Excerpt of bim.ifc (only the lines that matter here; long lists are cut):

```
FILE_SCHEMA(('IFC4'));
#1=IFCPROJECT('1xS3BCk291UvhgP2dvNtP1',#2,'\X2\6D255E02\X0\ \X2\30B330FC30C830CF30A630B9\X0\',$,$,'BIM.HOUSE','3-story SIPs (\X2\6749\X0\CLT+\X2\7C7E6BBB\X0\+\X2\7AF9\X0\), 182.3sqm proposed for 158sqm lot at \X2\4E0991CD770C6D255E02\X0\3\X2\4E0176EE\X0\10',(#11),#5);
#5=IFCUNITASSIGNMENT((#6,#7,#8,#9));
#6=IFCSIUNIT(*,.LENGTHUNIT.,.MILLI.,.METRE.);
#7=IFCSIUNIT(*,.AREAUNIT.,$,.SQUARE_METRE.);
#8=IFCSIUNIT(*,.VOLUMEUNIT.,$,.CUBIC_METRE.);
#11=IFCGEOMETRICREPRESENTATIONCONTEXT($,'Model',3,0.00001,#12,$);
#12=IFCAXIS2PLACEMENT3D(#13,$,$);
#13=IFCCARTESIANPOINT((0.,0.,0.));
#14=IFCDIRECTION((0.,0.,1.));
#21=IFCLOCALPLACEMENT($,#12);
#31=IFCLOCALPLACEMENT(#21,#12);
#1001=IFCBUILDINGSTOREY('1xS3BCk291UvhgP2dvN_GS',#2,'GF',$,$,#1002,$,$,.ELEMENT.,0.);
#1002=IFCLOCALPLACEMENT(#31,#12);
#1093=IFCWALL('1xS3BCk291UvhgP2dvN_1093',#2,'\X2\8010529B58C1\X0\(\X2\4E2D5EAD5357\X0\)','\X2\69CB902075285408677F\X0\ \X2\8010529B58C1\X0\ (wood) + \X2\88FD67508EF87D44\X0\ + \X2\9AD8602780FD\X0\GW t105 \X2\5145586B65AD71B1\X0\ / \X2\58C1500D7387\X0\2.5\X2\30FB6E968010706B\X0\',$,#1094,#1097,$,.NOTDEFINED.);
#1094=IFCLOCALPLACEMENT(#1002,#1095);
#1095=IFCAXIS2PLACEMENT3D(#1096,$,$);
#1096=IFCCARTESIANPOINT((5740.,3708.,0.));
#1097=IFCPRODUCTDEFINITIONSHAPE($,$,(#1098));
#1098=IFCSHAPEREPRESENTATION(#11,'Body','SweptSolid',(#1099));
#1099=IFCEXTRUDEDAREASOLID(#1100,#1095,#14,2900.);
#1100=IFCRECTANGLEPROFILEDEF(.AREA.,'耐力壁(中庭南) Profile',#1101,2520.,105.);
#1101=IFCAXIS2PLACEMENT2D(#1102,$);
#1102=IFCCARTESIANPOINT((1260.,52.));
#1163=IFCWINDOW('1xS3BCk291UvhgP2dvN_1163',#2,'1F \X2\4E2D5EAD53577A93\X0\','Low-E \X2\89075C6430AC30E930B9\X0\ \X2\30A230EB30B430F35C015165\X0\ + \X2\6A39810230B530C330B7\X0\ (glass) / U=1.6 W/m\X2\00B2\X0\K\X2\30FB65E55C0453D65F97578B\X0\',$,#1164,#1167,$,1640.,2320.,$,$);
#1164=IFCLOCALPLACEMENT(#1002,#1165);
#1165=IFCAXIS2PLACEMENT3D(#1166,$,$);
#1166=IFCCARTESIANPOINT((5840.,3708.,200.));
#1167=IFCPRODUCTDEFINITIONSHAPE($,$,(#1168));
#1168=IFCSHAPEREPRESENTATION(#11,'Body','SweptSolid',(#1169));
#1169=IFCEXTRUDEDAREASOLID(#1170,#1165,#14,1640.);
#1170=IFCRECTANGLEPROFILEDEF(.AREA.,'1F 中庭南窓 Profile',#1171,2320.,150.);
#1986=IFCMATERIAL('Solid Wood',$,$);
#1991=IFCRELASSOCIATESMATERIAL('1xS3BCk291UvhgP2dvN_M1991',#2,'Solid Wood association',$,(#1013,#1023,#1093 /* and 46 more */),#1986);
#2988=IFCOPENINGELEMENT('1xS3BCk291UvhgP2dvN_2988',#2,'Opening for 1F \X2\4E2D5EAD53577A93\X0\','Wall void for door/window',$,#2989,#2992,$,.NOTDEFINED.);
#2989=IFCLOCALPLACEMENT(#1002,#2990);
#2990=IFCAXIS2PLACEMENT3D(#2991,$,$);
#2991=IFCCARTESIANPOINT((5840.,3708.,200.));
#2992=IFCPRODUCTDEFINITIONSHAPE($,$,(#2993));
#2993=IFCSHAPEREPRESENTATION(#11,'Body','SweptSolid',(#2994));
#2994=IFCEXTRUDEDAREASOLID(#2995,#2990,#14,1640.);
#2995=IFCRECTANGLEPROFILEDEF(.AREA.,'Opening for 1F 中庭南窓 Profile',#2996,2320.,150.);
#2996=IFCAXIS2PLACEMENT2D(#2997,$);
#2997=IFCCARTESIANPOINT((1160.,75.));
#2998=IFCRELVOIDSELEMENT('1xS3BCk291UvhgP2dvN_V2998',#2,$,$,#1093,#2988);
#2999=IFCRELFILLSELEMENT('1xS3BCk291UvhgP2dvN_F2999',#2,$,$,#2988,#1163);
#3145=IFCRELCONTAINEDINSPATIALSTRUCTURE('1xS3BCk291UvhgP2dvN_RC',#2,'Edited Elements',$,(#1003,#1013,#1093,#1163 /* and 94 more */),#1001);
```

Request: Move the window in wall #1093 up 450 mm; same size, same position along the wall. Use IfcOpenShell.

```python
import numpy as np
import ifcopenshell
import ifcopenshell.api.geometry
import ifcopenshell.util.placement
import ifcopenshell.util.unit

model = ifcopenshell.open("bim.ifc")
unit_scale = ifcopenshell.util.unit.calculate_unit_scale(model)

window = model.by_id(1163)
opening = window.FillsVoids[0].RelatingOpeningElement
dz = 450.0

shift = np.array([0.0, 0.0, dz])
# The window is not placed relative to its opening, so move both.
for product in (opening, window):
    matrix = ifcopenshell.util.placement.get_local_placement(product.ObjectPlacement)
    matrix[:3, 3] += shift
    ifcopenshell.api.geometry.edit_object_placement(model, product=product, matrix=matrix, is_si=False)

print(f"moved by {dz * unit_scale:+.3f} m")

model.write("bim-out.ifc")
```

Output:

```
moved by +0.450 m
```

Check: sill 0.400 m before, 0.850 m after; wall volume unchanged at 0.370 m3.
